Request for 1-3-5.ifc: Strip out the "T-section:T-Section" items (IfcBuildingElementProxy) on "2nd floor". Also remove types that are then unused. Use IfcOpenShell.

First a look at what the model holds.

```python
import ifcopenshell
import ifcopenshell.util.element

model = ifcopenshell.open("1-3-5.ifc")
print(model.schema)
storey = next(s for s in model.by_type("IfcBuildingStorey") if s.Name == "2nd floor")
proxies = [e for e in ifcopenshell.util.element.get_decomposition(storey) if e.is_a("IfcBuildingElementProxy")]
seen = {}
for e in proxies:
    element_type = ifcopenshell.util.element.get_type(e)
    name = element_type.Name if element_type not in (None, e) else None
    seen[name] = seen.get(name, 0) + 1
for name, count in sorted(seen.items(), key=str):
    print(count, "x", name)
```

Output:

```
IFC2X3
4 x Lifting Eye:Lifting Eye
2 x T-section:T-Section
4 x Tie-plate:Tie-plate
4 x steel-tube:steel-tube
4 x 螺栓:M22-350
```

```python
import ifcopenshell
import ifcopenshell.api.root
import ifcopenshell.util.element

model = ifcopenshell.open("1-3-5.ifc")

storey = next(s for s in model.by_type("IfcBuildingStorey") if s.Name == "2nd floor")
proxies = [e for e in ifcopenshell.util.element.get_decomposition(storey) if e.is_a("IfcBuildingElementProxy")]
targets = [e for e in proxies if (t := ifcopenshell.util.element.get_type(e)) not in (None, e) and t.Name == "T-section:T-Section"]
types = {ifcopenshell.util.element.get_type(e) for e in targets} - {None, *targets}

for e in targets:
    ifcopenshell.api.root.remove_product(model, product=e)
print(len(targets), "removed")

unused = [t for t in types if not ifcopenshell.util.element.get_types(t)]
for t in unused:
    ifcopenshell.api.root.remove_product(model, product=t)
print(len(unused), "unused types removed")

model.write("1-3-5_updated.ifc")
```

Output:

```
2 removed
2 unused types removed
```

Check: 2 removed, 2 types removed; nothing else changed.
